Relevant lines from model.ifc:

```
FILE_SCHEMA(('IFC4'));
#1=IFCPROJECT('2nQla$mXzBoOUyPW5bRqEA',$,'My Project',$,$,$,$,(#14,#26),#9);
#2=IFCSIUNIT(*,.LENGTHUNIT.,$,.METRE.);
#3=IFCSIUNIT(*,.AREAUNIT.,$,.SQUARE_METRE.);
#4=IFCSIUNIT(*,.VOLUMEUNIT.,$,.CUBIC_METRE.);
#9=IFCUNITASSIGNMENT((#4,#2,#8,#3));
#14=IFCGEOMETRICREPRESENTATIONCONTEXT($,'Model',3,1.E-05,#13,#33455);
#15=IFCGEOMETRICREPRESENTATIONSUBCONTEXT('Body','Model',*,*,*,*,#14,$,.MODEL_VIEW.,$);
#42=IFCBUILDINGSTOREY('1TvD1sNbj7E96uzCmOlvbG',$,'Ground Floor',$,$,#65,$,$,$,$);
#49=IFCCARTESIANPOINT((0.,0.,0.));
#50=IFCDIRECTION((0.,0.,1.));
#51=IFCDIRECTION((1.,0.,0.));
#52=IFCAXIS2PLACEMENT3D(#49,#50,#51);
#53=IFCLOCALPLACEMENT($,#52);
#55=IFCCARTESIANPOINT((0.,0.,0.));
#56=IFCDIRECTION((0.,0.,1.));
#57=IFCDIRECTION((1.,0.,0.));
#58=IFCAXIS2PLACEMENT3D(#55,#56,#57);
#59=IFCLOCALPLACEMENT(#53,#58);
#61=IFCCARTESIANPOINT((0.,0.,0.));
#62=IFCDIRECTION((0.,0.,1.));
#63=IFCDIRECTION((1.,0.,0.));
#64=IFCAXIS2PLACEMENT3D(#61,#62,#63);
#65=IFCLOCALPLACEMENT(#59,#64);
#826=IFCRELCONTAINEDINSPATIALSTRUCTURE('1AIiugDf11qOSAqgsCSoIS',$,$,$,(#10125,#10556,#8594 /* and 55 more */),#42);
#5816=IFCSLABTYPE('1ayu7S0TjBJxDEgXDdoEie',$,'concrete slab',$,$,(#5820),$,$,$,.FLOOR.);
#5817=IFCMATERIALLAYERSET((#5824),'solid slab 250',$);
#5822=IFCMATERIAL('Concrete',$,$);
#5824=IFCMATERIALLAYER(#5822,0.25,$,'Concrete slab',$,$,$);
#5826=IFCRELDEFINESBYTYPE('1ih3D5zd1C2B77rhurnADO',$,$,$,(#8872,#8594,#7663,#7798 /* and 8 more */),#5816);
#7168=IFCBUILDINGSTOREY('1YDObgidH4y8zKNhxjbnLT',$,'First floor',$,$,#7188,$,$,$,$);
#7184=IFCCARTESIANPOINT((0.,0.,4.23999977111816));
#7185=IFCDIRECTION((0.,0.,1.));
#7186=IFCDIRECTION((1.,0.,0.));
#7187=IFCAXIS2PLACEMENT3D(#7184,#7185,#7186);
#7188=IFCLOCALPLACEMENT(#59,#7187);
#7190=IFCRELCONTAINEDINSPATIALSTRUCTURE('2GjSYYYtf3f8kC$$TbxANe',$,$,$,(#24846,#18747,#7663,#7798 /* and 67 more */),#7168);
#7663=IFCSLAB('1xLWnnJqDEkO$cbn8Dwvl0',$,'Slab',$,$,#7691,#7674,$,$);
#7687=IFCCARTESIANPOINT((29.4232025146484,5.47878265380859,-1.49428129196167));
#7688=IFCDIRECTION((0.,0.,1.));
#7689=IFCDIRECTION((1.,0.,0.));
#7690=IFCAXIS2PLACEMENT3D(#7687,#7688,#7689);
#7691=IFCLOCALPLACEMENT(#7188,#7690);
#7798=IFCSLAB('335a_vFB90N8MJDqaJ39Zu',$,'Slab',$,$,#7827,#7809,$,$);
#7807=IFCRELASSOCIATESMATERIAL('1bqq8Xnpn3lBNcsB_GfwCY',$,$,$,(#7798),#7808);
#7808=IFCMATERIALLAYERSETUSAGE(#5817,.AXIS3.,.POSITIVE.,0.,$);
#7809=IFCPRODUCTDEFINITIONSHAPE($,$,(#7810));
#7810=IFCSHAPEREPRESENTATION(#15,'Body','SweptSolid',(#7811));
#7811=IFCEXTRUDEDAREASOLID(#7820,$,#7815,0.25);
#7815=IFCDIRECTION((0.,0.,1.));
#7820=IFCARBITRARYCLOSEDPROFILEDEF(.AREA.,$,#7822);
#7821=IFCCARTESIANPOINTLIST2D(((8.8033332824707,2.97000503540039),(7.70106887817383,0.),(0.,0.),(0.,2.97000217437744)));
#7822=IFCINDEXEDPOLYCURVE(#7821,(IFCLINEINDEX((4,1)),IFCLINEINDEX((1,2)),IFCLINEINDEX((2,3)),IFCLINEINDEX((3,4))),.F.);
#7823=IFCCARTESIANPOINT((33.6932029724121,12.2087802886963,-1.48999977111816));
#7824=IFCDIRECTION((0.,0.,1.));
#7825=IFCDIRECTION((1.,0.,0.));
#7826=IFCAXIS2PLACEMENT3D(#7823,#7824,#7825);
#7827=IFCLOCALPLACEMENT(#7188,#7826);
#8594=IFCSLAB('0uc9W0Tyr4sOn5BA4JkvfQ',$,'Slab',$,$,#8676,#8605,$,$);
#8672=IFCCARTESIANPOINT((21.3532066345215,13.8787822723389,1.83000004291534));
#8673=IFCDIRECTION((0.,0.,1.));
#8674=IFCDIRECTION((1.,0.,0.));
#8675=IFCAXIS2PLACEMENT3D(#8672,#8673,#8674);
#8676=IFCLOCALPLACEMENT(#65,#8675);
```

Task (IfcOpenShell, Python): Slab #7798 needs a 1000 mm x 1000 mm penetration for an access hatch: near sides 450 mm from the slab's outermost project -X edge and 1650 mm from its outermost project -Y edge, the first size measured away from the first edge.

```python
import numpy as np
import ifcopenshell
import ifcopenshell.api.feature
import ifcopenshell.api.geometry
import ifcopenshell.api.root
import ifcopenshell.geom
import ifcopenshell.util.placement
import ifcopenshell.util.representation
import ifcopenshell.util.shape
import ifcopenshell.util.unit

model = ifcopenshell.open("model.ifc")
unit_scale = ifcopenshell.util.unit.calculate_unit_scale(model)
settings = ifcopenshell.geom.settings()


def volume(element):
    """Net volume in cubic metres, openings subtracted."""
    shape = ifcopenshell.geom.create_shape(settings, element)
    return ifcopenshell.util.shape.get_volume(shape.geometry)


slab = model.by_id(7798)
before = volume(slab)

# Extent in the slab's own axes, in metres. The edges named are its -X and -Y sides.
slab_shape = ifcopenshell.geom.create_shape(settings, slab)
vertices = ifcopenshell.util.shape.get_vertices(slab_shape.geometry)
x_min, y_min, bottom = vertices.min(axis=0)
top = vertices[:, 2].max()

opening = ifcopenshell.api.root.create_entity(model, ifc_class="IfcOpeningElement", name="Access hatch opening", predefined_type="OPENING")
context = ifcopenshell.util.representation.get_context(model, "Model", "Body", "MODEL_VIEW")
width, depth = 1, 1
outline = [(0.0, 0.0), (width, 0.0), (width, depth), (0.0, depth), (0.0, 0.0)]
# Overshoot both faces by 50 mm so the cut is clean.
shape = ifcopenshell.api.geometry.add_slab_representation(
    model, context=context, depth=top - bottom + 0.1, polyline=outline
)
ifcopenshell.api.geometry.assign_representation(model, product=opening, representation=shape)

matrix = ifcopenshell.util.placement.get_local_placement(slab.ObjectPlacement)
matrix[:, 3] = matrix @ np.append(np.array([x_min + 0.45, y_min + 1.65, bottom - 0.05]) / unit_scale, 1.0)
ifcopenshell.api.geometry.edit_object_placement(model, product=opening, matrix=matrix, is_si=False)
ifcopenshell.api.feature.add_feature(model, feature=opening, element=slab)

after = volume(slab)

print(f"slab volume {before:.3f} -> {after:.3f} m3")

model.write("model_edited.ifc")
```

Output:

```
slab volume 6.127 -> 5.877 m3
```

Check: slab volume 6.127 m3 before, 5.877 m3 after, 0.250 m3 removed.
